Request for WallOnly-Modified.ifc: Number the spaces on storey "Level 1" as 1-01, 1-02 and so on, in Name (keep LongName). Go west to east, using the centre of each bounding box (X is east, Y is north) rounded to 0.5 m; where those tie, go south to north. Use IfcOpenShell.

First a look at what the model holds.

```python
import ifcopenshell
import ifcopenshell.util.element
import ifcopenshell.util.placement

model = ifcopenshell.open("WallOnly-Modified.ifc")
print(model.schema)
storey = next(s for s in model.by_type("IfcBuildingStorey") if s.Name == "Level 1")
spaces = [e for e in ifcopenshell.util.element.get_decomposition(storey) if e.is_a("IfcSpace")]
for e in sorted(spaces, key=lambda e: e.id()):
    origin = ifcopenshell.util.placement.get_local_placement(e.ObjectPlacement)[:3, 3]
    print(e.id(), e.Name, e.LongName, origin.round(2) + 0.0, sep=" | ")
```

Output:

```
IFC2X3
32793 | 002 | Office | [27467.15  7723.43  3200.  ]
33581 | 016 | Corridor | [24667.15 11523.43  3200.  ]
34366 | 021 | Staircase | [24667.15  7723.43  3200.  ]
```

```python
import ifcopenshell
import ifcopenshell.geom
import ifcopenshell.util.element
import ifcopenshell.util.shape

model = ifcopenshell.open("WallOnly-Modified.ifc")
settings = ifcopenshell.geom.settings()
settings.set("use-world-coords", True)


def centre(element):
    shape = ifcopenshell.geom.create_shape(settings, element)
    return ifcopenshell.util.shape.get_bbox_centroid(shape.geometry)


storey = next(s for s in model.by_type("IfcBuildingStorey") if s.Name == "Level 1")
spaces = [e for e in ifcopenshell.util.element.get_decomposition(storey) if e.is_a("IfcSpace")]

# Insertion points can sit at a corner or the storey origin, so sort by the geometry (in metres).
centres = {e: centre(e) for e in spaces}
spaces.sort(key=lambda e: (round(centres[e][0] / 0.5), centres[e][1]))

for i, e in enumerate(spaces, start=1):
    number = f"1-{i:02d}"
    e.Name = number
    print(e.id(), number)

model.write("WallOnly-Modified_edited.ifc")
```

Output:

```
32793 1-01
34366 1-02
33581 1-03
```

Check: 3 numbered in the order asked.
